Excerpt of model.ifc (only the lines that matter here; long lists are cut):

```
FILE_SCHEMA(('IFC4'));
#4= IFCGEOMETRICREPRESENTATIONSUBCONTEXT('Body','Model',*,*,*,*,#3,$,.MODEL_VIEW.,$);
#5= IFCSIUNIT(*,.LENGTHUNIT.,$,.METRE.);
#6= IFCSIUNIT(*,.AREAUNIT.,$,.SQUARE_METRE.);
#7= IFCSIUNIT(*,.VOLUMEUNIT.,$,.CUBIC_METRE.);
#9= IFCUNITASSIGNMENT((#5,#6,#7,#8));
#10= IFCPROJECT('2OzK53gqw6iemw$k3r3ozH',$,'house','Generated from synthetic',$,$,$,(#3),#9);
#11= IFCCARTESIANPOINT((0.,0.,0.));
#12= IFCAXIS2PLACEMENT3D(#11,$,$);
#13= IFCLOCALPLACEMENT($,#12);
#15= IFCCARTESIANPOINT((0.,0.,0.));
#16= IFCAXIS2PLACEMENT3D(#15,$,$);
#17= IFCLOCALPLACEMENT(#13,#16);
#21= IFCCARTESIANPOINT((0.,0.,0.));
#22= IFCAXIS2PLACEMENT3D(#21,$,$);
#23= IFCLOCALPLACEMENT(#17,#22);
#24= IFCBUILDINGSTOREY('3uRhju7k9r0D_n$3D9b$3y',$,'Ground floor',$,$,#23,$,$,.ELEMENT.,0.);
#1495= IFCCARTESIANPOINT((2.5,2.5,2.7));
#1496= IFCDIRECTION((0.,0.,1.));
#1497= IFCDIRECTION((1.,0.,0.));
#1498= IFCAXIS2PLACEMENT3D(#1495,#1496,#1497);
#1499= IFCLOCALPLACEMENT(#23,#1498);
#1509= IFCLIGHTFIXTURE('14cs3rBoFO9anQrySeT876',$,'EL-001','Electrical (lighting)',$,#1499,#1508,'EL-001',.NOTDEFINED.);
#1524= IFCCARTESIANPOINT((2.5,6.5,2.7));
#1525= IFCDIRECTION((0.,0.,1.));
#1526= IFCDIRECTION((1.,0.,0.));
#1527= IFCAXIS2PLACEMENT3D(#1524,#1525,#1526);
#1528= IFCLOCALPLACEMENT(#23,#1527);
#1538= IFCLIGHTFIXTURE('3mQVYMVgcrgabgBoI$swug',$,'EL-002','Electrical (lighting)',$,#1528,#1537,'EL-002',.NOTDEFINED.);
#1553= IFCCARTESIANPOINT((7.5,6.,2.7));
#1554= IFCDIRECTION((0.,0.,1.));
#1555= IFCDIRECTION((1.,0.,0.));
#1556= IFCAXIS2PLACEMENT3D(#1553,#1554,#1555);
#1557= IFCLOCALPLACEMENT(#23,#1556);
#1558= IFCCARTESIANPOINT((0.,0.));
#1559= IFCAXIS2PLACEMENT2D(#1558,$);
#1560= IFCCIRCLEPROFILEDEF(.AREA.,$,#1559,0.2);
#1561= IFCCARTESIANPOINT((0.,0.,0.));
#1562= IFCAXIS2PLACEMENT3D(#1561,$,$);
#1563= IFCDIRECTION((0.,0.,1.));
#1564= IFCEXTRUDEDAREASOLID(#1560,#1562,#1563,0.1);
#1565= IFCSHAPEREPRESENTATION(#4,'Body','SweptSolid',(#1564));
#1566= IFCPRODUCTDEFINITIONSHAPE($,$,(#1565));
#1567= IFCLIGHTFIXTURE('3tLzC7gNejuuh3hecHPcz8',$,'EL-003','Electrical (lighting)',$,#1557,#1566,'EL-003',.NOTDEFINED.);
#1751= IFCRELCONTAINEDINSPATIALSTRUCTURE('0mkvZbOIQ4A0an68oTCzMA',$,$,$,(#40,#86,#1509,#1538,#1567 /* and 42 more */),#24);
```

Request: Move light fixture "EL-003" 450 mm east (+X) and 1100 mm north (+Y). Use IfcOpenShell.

```python
import ifcopenshell
import ifcopenshell.api.geometry
import ifcopenshell.util.placement

model = ifcopenshell.open("model.ifc")

item = model.by_guid("3tLzC7gNejuuh3hecHPcz8")
matrix = ifcopenshell.util.placement.get_local_placement(item.ObjectPlacement)
matrix[0, 3] += 0.45
matrix[1, 3] += 1.1
ifcopenshell.api.geometry.edit_object_placement(model, product=item, matrix=matrix, is_si=False)

print(ifcopenshell.util.placement.get_local_placement(item.ObjectPlacement).round(3) + 0.0)

model.write("model_rev.ifc")
```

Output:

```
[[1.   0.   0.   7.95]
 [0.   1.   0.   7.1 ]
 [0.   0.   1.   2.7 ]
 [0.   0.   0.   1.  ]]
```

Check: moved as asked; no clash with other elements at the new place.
